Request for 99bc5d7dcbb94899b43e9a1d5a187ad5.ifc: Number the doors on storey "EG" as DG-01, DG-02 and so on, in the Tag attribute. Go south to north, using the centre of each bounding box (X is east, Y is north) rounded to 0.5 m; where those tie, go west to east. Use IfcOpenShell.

First a look at what the model holds.

```python
import ifcopenshell
import ifcopenshell.util.element
import ifcopenshell.util.placement

model = ifcopenshell.open("99bc5d7dcbb94899b43e9a1d5a187ad5.ifc")
print(model.schema)
storey = next(s for s in model.by_type("IfcBuildingStorey") if s.Name == "EG")
doors = [e for e in ifcopenshell.util.element.get_decomposition(storey) if e.is_a("IfcDoor")]
for e in sorted(doors, key=lambda e: e.id()):
    origin = ifcopenshell.util.placement.get_local_placement(e.ObjectPlacement)[:3, 3]
    print(e.id(), e.Tag, e.Name, origin.round(2) + 0.0, sep=" | ")
```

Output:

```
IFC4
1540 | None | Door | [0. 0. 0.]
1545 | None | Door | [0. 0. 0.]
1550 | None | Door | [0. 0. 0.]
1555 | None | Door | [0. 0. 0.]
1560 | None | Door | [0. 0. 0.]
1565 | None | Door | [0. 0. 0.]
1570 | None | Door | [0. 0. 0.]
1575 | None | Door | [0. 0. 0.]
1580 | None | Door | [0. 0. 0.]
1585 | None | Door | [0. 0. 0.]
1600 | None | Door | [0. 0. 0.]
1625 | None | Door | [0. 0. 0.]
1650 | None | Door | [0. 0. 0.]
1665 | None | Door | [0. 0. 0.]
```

```python
import ifcopenshell
import ifcopenshell.geom
import ifcopenshell.util.element
import ifcopenshell.util.shape

model = ifcopenshell.open("99bc5d7dcbb94899b43e9a1d5a187ad5.ifc")
settings = ifcopenshell.geom.settings()
settings.set("use-world-coords", True)


def centre(element):
    shape = ifcopenshell.geom.create_shape(settings, element)
    return ifcopenshell.util.shape.get_bbox_centroid(shape.geometry)


storey = next(s for s in model.by_type("IfcBuildingStorey") if s.Name == "EG")
doors = [e for e in ifcopenshell.util.element.get_decomposition(storey) if e.is_a("IfcDoor")]

# Insertion points can sit at a corner or the storey origin, so sort by the geometry (in metres).
centres = {e: centre(e) for e in doors}
doors.sort(key=lambda e: (round(centres[e][1] / 0.5), centres[e][0]))

for i, e in enumerate(doors, start=1):
    number = f"DG-{i:02d}"
    e.Tag = number
    print(e.id(), number)

model.write("99bc5d7dcbb94899b43e9a1d5a187ad5_updated.ifc")
```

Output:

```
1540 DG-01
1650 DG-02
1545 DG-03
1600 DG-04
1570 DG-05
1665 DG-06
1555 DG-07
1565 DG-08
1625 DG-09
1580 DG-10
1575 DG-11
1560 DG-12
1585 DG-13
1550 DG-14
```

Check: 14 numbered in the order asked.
